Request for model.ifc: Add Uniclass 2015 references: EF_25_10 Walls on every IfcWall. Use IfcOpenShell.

First a look at what the model holds.

```python
import ifcopenshell

model = ifcopenshell.open("model.ifc")
print(model.schema)
print("classifications:", [c.Name for c in model.by_type("IfcClassification")])
for ifc_class in ("IfcDoor", "IfcRoof", "IfcStair", "IfcWall", "IfcWindow"):
    print(ifc_class, len(model.by_type(ifc_class)))
```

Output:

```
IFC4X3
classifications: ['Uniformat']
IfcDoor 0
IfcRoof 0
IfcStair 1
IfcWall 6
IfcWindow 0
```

```python
import ifcopenshell
import ifcopenshell.api.classification

model = ifcopenshell.open("model.ifc")

system = ifcopenshell.api.classification.add_classification(model, classification="Uniclass 2015")

codes = {
    "IfcWall": ("EF_25_10", "Walls"),
}
for ifc_class, (code, name) in codes.items():
    products = model.by_type(ifc_class)
    ifcopenshell.api.classification.add_reference(
        model, products=products, classification=system, identification=code, name=name
    )
    print(code, len(products))

model.write("model-out.ifc")
```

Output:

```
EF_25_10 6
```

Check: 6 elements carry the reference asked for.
